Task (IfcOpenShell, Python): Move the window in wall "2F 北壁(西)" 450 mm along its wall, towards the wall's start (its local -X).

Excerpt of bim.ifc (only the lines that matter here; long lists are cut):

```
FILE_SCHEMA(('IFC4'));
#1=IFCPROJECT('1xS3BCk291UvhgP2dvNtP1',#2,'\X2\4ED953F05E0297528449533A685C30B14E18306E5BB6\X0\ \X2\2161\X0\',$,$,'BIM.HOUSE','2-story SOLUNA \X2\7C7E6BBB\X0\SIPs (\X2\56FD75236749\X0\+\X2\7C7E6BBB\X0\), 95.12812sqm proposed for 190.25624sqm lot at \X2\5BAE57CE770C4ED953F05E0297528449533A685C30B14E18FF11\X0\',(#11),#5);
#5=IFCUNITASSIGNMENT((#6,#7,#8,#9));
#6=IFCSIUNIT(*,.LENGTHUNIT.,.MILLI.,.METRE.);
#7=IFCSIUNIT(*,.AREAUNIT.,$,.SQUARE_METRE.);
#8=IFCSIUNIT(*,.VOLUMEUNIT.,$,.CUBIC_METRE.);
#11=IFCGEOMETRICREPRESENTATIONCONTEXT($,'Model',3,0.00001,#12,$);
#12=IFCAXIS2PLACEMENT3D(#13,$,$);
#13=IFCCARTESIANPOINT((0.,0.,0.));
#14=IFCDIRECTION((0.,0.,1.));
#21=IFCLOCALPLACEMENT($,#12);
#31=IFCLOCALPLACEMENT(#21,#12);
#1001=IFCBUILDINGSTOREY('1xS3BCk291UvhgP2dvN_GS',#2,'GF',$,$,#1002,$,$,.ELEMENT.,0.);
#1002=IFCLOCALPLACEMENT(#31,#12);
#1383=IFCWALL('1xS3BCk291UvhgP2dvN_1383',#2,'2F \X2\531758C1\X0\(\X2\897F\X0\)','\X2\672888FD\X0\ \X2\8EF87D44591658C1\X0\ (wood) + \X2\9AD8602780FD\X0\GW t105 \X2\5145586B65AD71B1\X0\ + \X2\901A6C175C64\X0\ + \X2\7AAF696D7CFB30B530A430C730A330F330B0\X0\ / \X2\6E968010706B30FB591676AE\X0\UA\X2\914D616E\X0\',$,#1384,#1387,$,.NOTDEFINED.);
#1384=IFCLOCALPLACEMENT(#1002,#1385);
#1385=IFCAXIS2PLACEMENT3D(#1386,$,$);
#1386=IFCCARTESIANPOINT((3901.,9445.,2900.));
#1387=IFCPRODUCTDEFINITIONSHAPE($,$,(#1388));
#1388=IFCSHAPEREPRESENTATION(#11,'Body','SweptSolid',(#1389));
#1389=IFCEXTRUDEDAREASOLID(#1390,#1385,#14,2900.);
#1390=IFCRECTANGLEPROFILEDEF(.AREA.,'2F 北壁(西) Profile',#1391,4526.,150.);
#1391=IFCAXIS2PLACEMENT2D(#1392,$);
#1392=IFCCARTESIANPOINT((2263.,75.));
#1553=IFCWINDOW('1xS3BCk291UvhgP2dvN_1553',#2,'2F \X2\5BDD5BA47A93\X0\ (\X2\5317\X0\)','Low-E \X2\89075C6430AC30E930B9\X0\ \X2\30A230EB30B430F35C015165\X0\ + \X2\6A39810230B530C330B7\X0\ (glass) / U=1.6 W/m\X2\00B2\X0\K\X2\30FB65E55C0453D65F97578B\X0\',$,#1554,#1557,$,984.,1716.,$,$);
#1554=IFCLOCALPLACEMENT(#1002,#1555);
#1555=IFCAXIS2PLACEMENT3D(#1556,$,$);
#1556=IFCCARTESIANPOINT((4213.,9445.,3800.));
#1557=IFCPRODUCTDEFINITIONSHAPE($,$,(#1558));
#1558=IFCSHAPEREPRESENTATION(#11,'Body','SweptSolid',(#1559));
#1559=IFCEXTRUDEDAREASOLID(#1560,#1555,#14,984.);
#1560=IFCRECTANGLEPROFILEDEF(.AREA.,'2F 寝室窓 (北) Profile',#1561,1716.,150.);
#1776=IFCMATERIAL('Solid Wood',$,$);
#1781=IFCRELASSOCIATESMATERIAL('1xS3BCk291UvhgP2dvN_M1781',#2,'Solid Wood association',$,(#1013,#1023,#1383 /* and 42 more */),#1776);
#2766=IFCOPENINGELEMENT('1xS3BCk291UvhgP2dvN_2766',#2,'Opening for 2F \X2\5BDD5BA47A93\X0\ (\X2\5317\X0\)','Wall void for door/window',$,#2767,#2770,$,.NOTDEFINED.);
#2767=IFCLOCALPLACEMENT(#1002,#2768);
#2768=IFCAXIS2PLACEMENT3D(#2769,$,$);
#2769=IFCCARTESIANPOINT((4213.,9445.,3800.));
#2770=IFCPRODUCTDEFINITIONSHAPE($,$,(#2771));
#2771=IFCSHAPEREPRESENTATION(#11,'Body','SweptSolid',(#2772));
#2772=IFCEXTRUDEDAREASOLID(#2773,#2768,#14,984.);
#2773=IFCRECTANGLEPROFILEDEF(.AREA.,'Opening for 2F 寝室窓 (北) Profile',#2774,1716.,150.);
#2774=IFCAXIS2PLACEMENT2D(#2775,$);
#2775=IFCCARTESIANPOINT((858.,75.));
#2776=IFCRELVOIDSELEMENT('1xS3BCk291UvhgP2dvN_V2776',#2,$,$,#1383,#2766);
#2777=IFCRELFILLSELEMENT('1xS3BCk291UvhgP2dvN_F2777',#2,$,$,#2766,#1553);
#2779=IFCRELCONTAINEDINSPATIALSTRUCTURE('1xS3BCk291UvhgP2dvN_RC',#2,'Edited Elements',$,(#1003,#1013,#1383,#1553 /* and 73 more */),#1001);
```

```python
import ifcopenshell
import ifcopenshell.api.geometry
import ifcopenshell.util.placement

model = ifcopenshell.open("bim.ifc")

window = model.by_guid("1xS3BCk291UvhgP2dvN_1553")
opening = window.FillsVoids[0].RelatingOpeningElement
wall = opening.VoidsElements[0].RelatingBuildingElement

wall_matrix = ifcopenshell.util.placement.get_local_placement(wall.ObjectPlacement)
shift = wall_matrix[:3, 0] * -450.0
before = ifcopenshell.util.placement.get_local_placement(window.ObjectPlacement)[:3, 3].copy()

# The window is not placed relative to its opening, so move both.
for product in (opening, window):
    matrix = ifcopenshell.util.placement.get_local_placement(product.ObjectPlacement)
    matrix[:3, 3] += shift
    ifcopenshell.api.geometry.edit_object_placement(model, product=product, matrix=matrix, is_si=False)

after = ifcopenshell.util.placement.get_local_placement(window.ObjectPlacement)[:3, 3]
print("window moved by", (after - before).round(3) + 0.0)

model.write("bim_rev.ifc")
```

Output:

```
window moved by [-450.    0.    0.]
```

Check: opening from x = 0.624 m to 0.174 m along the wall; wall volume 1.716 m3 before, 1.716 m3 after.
